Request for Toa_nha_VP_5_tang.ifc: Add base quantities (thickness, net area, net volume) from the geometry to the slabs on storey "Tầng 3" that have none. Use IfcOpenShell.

First a look at what the model holds.

```python
import ifcopenshell
import ifcopenshell.util.element
import ifcopenshell.util.unit

model = ifcopenshell.open("Toa_nha_VP_5_tang.ifc")
print(model.schema)
for unit_type in ("LENGTHUNIT", "AREAUNIT", "VOLUMEUNIT"):
    print(unit_type, ifcopenshell.util.unit.calculate_unit_scale(model, unit_type))
storey = next(s for s in model.by_type("IfcBuildingStorey") if s.Name == "Tầng 3")
slabs = [e for e in ifcopenshell.util.element.get_decomposition(storey) if e.is_a("IfcSlab")]
for e in sorted(slabs, key=lambda e: e.id()):
    print(e.id(), e.is_a(), e.Name, list(ifcopenshell.util.element.get_psets(e, qtos_only=True)), sep=" | ")
```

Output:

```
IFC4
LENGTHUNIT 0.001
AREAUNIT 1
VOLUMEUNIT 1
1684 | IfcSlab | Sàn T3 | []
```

```python
import ifcopenshell
import ifcopenshell.api.pset
import ifcopenshell.geom
import ifcopenshell.util.element
import ifcopenshell.util.shape
import ifcopenshell.util.unit

model = ifcopenshell.open("Toa_nha_VP_5_tang.ifc")
unit_scale = ifcopenshell.util.unit.calculate_unit_scale(model)
area_scale = ifcopenshell.util.unit.calculate_unit_scale(model, "AREAUNIT")
volume_scale = ifcopenshell.util.unit.calculate_unit_scale(model, "VOLUMEUNIT")
settings = ifcopenshell.geom.settings()

storey = next(s for s in model.by_type("IfcBuildingStorey") if s.Name == "Tầng 3")
slabs = [e for e in ifcopenshell.util.element.get_decomposition(storey) if e.is_a("IfcSlab")]

for e in sorted(slabs, key=lambda e: e.id()):
    if ifcopenshell.util.element.get_psets(e, qtos_only=True, should_inherit=False):
        continue
    # Geometry comes back in metres, in the element's own axes.
    shape = ifcopenshell.geom.create_shape(settings, e)
    values = {
        "Width": ifcopenshell.util.shape.get_z(shape.geometry) / unit_scale,
        "NetArea": ifcopenshell.util.shape.get_footprint_area(shape.geometry) / area_scale,
        "NetVolume": ifcopenshell.util.shape.get_volume(shape.geometry) / volume_scale,
    }
    qto = ifcopenshell.api.pset.add_qto(model, product=e, name="Qto_SlabBaseQuantities")
    ifcopenshell.api.pset.edit_qto(model, qto=qto, properties=values)
    print(e.id(), {k: round(v, 3) for k, v in values.items()})

model.write("Toa_nha_VP_5_tang_rev.ifc")
```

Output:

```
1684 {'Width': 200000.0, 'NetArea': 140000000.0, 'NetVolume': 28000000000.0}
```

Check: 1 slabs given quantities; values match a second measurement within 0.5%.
